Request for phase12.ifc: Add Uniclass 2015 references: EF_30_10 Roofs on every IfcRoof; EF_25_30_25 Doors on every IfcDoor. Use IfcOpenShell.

First a look at what the model holds.

```python
import ifcopenshell

model = ifcopenshell.open("phase12.ifc")
print(model.schema)
print("classifications:", [c.Name for c in model.by_type("IfcClassification")])
for ifc_class in ("IfcDoor", "IfcRoof", "IfcStair", "IfcWall", "IfcWindow"):
    print(ifc_class, len(model.by_type(ifc_class)))
```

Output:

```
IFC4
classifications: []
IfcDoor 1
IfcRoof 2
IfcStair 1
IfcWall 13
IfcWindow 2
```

```python
import ifcopenshell
import ifcopenshell.api.classification

model = ifcopenshell.open("phase12.ifc")

system = ifcopenshell.api.classification.add_classification(model, classification="Uniclass 2015")

codes = {
    "IfcRoof": ("EF_30_10", "Roofs"),
    "IfcDoor": ("EF_25_30_25", "Doors"),
}
for ifc_class, (code, name) in codes.items():
    products = model.by_type(ifc_class)
    ifcopenshell.api.classification.add_reference(
        model, products=products, classification=system, identification=code, name=name
    )
    print(code, len(products))

model.write("phase12_edited.ifc")
```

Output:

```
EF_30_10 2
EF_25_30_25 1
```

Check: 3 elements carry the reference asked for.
